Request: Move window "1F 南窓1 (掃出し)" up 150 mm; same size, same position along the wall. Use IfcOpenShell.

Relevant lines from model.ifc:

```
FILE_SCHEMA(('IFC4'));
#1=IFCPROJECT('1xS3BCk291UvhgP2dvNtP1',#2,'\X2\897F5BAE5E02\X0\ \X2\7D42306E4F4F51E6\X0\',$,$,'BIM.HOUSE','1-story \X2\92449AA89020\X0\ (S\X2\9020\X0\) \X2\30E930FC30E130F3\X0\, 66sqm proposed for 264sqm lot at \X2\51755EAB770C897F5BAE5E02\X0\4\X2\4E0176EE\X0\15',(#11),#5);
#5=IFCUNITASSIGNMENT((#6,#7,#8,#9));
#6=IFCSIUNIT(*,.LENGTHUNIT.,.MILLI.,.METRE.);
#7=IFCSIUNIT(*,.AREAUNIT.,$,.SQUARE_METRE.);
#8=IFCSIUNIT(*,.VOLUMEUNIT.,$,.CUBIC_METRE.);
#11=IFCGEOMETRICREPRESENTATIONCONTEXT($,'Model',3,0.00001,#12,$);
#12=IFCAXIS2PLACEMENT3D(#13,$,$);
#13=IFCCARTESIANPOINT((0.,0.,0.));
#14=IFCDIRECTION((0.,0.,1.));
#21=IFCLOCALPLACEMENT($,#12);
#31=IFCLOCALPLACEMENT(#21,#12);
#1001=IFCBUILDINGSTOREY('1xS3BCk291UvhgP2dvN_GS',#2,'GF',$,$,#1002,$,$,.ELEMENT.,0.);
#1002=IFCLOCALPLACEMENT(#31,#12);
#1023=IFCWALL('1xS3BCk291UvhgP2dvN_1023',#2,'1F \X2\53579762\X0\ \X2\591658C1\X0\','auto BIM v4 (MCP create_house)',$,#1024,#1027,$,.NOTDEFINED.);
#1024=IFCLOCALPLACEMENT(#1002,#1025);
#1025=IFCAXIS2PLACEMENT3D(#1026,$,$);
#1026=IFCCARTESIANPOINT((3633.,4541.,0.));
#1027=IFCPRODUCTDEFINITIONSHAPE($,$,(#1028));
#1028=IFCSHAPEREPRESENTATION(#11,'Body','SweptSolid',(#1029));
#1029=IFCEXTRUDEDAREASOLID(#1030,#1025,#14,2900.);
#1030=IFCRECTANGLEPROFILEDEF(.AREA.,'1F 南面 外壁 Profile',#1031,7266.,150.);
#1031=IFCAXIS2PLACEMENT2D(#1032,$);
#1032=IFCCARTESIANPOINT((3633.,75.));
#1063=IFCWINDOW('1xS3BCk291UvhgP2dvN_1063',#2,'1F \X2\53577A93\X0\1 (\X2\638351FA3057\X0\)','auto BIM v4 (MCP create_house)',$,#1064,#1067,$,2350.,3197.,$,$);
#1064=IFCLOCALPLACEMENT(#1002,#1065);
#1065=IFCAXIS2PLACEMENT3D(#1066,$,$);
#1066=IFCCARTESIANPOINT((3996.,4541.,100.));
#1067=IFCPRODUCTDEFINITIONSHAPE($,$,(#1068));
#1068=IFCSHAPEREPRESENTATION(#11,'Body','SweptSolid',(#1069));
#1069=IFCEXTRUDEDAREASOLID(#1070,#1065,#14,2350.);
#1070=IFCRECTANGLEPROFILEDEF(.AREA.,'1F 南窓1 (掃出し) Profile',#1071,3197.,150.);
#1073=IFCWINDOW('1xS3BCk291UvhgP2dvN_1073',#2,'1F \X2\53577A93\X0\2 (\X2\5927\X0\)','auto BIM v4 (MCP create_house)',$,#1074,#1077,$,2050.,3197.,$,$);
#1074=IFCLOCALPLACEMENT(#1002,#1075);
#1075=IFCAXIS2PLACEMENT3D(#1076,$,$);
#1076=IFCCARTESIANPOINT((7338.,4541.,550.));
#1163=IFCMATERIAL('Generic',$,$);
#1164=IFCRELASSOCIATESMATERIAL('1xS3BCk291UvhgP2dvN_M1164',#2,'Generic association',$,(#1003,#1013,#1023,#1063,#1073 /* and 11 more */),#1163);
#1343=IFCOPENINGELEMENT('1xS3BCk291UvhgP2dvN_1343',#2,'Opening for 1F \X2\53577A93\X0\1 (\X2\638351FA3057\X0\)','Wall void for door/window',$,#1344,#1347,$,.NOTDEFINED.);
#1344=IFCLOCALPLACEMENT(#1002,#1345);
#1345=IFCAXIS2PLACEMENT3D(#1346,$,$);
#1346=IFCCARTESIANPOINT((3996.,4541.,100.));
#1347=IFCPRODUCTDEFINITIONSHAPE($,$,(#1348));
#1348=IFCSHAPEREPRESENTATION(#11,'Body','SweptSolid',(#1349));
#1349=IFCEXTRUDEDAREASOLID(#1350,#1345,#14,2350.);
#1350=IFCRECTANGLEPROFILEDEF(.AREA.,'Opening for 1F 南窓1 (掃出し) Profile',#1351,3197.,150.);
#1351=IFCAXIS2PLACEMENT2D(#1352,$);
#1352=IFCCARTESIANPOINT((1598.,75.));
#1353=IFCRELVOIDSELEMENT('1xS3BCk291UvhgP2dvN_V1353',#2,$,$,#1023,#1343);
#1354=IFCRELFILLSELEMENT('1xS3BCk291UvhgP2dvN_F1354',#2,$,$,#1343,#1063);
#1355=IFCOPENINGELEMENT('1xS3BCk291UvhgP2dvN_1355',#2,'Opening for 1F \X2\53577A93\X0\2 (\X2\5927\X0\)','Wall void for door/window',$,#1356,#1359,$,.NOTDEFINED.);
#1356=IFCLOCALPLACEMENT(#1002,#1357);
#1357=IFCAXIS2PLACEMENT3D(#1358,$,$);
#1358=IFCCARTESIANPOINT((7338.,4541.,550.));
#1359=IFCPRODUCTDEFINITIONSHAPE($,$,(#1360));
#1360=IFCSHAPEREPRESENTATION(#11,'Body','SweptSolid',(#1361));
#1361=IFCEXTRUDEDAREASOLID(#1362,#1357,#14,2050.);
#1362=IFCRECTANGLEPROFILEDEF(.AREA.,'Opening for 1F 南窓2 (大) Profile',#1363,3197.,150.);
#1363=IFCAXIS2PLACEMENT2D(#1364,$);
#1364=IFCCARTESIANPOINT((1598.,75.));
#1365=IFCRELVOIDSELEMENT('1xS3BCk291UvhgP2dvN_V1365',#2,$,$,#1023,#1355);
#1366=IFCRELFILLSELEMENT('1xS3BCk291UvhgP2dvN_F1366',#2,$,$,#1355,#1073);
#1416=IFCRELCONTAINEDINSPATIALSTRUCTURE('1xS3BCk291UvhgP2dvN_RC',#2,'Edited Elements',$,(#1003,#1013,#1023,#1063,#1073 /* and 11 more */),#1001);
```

```python
import numpy as np
import ifcopenshell
import ifcopenshell.api.geometry
import ifcopenshell.util.placement
import ifcopenshell.util.unit

model = ifcopenshell.open("model.ifc")
unit_scale = ifcopenshell.util.unit.calculate_unit_scale(model)

window = model.by_guid("1xS3BCk291UvhgP2dvN_1063")
opening = window.FillsVoids[0].RelatingOpeningElement
dz = 150.0

shift = np.array([0.0, 0.0, dz])
# The window is not placed relative to its opening, so move both.
for product in (opening, window):
    matrix = ifcopenshell.util.placement.get_local_placement(product.ObjectPlacement)
    matrix[:3, 3] += shift
    ifcopenshell.api.geometry.edit_object_placement(model, product=product, matrix=matrix, is_si=False)

print(f"moved by {dz * unit_scale:+.3f} m")

model.write("model_updated.ifc")
```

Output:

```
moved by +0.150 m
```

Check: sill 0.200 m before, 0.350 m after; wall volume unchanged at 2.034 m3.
